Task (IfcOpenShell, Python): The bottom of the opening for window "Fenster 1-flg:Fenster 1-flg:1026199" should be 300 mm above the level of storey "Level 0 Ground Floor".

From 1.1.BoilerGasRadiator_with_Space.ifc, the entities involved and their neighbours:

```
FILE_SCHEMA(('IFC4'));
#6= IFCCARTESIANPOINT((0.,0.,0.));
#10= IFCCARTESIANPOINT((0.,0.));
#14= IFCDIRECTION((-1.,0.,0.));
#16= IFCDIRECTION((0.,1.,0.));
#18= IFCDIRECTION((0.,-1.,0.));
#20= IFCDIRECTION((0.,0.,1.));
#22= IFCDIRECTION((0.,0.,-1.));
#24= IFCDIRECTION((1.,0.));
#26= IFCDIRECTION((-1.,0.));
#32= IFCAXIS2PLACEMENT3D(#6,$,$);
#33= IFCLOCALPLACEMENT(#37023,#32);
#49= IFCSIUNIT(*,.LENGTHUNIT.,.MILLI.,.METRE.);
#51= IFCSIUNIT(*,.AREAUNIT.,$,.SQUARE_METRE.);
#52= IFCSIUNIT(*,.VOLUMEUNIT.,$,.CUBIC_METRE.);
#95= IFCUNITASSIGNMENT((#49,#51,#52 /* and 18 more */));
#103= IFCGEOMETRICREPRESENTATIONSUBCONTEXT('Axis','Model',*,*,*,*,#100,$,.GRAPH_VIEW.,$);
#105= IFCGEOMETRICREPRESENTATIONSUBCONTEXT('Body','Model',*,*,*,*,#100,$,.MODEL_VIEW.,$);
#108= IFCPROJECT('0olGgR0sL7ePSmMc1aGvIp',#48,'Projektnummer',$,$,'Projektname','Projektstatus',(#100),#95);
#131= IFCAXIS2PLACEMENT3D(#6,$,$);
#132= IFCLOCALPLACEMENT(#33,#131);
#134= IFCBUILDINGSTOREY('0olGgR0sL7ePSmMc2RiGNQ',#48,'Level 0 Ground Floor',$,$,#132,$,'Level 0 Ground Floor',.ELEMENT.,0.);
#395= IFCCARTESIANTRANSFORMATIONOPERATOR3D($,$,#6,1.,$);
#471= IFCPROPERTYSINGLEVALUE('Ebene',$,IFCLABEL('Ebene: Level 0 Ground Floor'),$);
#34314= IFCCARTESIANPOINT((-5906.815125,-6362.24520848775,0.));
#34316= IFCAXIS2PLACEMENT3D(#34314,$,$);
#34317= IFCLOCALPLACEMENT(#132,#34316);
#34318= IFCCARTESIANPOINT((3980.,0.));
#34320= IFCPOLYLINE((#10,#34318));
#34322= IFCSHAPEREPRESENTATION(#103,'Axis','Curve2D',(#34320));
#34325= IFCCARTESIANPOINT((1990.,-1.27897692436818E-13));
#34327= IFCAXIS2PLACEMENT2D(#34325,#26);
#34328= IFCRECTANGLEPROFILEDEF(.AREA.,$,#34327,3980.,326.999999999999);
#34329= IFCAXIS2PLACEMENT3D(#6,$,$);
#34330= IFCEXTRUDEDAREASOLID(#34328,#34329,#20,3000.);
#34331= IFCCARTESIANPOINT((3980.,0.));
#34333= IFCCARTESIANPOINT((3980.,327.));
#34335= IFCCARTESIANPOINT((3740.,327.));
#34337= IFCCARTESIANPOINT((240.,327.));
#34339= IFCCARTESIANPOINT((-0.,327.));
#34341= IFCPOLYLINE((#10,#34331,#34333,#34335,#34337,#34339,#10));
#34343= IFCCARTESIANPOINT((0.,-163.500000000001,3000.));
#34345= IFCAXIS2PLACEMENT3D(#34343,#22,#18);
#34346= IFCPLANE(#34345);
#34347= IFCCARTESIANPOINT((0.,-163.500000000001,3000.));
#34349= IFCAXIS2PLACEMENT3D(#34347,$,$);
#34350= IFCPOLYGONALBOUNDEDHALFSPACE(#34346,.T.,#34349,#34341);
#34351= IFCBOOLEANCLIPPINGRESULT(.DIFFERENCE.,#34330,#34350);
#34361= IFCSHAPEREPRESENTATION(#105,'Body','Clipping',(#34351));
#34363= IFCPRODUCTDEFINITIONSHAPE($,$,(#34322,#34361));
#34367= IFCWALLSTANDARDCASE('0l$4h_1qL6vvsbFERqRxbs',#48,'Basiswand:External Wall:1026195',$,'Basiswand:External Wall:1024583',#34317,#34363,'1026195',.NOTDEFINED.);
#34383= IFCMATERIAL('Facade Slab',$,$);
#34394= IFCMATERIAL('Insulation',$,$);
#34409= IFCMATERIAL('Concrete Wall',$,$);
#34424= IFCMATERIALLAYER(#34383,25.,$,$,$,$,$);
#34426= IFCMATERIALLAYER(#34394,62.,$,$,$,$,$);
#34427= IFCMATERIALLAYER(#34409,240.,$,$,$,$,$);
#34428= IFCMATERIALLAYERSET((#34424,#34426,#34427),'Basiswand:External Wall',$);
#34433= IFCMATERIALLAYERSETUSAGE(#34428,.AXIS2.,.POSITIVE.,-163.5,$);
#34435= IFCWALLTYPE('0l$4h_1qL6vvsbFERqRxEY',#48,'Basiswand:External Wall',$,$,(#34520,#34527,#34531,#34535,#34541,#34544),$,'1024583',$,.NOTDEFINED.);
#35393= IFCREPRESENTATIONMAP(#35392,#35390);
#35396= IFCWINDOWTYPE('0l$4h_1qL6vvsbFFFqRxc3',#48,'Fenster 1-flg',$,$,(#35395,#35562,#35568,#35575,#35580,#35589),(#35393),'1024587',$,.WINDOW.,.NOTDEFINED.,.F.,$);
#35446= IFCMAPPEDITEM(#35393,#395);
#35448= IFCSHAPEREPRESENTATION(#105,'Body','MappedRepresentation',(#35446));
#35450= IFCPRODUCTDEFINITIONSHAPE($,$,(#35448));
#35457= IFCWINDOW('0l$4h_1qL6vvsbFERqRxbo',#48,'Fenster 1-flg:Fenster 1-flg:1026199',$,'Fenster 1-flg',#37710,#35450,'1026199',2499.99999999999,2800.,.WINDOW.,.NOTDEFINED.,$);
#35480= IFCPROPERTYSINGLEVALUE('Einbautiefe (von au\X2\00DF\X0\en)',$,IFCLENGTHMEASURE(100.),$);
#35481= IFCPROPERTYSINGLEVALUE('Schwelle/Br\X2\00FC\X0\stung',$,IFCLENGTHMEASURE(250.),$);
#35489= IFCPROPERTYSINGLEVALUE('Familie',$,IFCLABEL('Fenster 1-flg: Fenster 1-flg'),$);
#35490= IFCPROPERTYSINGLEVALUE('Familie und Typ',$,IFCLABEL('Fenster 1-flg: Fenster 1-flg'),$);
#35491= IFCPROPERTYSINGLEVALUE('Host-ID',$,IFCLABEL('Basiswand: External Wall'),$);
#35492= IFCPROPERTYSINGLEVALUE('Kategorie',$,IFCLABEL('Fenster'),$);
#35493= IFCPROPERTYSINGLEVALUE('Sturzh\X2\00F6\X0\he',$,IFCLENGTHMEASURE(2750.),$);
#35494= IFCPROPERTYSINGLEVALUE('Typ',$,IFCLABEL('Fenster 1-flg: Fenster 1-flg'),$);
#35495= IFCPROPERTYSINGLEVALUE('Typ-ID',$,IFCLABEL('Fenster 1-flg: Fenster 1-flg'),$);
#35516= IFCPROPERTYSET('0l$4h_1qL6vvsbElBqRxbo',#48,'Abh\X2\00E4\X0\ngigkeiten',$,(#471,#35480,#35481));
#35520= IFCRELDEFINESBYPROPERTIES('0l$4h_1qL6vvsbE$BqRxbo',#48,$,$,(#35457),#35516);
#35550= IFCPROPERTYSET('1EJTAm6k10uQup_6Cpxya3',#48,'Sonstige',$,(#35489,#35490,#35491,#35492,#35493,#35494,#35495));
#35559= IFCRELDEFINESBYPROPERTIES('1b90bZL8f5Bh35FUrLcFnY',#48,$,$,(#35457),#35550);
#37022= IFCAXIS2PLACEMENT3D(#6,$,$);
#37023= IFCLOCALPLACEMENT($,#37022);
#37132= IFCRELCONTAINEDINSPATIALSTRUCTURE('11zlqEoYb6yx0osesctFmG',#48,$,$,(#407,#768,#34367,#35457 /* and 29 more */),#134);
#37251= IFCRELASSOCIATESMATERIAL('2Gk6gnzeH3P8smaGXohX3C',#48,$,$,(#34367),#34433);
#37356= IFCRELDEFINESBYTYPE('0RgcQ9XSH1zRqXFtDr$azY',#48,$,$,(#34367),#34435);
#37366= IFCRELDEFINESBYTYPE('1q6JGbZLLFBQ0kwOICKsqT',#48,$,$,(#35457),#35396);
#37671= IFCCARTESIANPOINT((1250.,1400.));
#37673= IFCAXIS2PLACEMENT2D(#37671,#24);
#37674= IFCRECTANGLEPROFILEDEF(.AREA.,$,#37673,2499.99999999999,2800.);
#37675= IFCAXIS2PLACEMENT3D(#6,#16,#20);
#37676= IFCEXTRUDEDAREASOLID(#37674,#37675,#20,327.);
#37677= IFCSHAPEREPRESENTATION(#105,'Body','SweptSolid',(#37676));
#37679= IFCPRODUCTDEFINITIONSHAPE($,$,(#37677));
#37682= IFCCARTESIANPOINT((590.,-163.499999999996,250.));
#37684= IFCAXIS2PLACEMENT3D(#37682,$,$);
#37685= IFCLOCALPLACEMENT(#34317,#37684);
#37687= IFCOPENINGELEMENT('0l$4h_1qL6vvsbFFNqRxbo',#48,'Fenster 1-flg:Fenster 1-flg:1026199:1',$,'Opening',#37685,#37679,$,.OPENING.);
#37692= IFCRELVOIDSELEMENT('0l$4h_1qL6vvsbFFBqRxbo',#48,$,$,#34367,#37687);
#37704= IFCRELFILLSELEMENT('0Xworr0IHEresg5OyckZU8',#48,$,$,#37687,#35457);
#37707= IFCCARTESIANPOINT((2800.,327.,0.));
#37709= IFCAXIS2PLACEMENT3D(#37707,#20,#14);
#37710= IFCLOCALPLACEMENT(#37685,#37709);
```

```python
import numpy as np
import ifcopenshell
import ifcopenshell.api.geometry
import ifcopenshell.api.pset
import ifcopenshell.geom
import ifcopenshell.util.element
import ifcopenshell.util.placement
import ifcopenshell.util.shape
import ifcopenshell.util.unit

model = ifcopenshell.open("1.1.BoilerGasRadiator_with_Space.ifc")
unit_scale = ifcopenshell.util.unit.calculate_unit_scale(model)

window = model.by_guid("0l$4h_1qL6vvsbFERqRxbo")
opening = window.FillsVoids[0].RelatingOpeningElement
storey = ifcopenshell.util.element.get_container(window, ifc_class="IfcBuildingStorey")
level = ifcopenshell.util.placement.get_local_placement(storey.ObjectPlacement)[2, 3]

# The opening's origin need not be at the sill, so measure its lowest point.
shape = ifcopenshell.geom.create_shape(ifcopenshell.geom.settings(), opening)
bottom = ifcopenshell.util.shape.get_shape_bottom_elevation(shape, shape.geometry) / unit_scale
dz = level + 0.3 / unit_scale - bottom

shift = np.array([0.0, 0.0, dz])
# The window is placed relative to its opening, so it follows when the opening moves.
matrix = ifcopenshell.util.placement.get_local_placement(opening.ObjectPlacement)
matrix[:3, 3] += shift
ifcopenshell.api.geometry.edit_object_placement(
    model, product=opening, matrix=matrix, is_si=False, should_transform_children=True
)

# Keep the stored heights in step.
pset = model.by_id(ifcopenshell.util.element.get_pset(window, "Abhängigkeiten", should_inherit=False)["id"])
ifcopenshell.api.pset.edit_pset(model, pset=pset, properties={
    "Schwelle/Brüstung": model.create_entity("IfcLengthMeasure", ifcopenshell.util.element.get_pset(window, "Abhängigkeiten", "Schwelle/Brüstung") + dz),
})
pset = model.by_id(ifcopenshell.util.element.get_pset(window, "Sonstige", should_inherit=False)["id"])
ifcopenshell.api.pset.edit_pset(model, pset=pset, properties={
    "Sturzhöhe": model.create_entity("IfcLengthMeasure", ifcopenshell.util.element.get_pset(window, "Sonstige", "Sturzhöhe") + dz),
})

print(f"moved by {dz * unit_scale:+.3f} m")

model.write("1.1.BoilerGasRadiator_with_Space_rev.ifc")
```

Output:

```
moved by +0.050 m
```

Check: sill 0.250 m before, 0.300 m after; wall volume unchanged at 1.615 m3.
